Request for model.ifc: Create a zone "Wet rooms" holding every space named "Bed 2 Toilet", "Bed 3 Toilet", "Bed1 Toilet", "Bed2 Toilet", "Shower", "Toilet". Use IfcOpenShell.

First a look at what the model holds.

```python
import ifcopenshell

model = ifcopenshell.open("model.ifc")
print(model.schema)
seen = {}
for space in model.by_type("IfcSpace"):
    seen[space.Name] = seen.get(space.Name, 0) + 1
for name, count in sorted(seen.items(), key=str):
    print(count, "x", name)
print("zones:", [z.Name for z in model.by_type("IfcZone")][:20])
```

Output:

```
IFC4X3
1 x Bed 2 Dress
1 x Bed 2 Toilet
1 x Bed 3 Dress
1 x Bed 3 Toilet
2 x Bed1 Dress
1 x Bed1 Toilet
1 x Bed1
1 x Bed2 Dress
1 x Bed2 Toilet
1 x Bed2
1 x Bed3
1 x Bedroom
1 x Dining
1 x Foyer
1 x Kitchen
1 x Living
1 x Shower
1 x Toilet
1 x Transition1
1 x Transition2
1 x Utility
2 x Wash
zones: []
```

```python
import ifcopenshell
import ifcopenshell.api.group
import ifcopenshell.api.root

model = ifcopenshell.open("model.ifc")

names = {"Bed 2 Toilet", "Bed 3 Toilet", "Bed1 Toilet", "Bed2 Toilet", "Shower", "Toilet"}
spaces = [s for s in model.by_type("IfcSpace") if s.Name in names]

zone = ifcopenshell.api.root.create_entity(model, ifc_class="IfcZone", name="Wet rooms")
ifcopenshell.api.group.assign_group(model, products=spaces, group=zone)
print(len(spaces), "spaces in", zone.Name)

model.write("model_updated.ifc")
```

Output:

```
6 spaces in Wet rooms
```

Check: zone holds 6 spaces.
